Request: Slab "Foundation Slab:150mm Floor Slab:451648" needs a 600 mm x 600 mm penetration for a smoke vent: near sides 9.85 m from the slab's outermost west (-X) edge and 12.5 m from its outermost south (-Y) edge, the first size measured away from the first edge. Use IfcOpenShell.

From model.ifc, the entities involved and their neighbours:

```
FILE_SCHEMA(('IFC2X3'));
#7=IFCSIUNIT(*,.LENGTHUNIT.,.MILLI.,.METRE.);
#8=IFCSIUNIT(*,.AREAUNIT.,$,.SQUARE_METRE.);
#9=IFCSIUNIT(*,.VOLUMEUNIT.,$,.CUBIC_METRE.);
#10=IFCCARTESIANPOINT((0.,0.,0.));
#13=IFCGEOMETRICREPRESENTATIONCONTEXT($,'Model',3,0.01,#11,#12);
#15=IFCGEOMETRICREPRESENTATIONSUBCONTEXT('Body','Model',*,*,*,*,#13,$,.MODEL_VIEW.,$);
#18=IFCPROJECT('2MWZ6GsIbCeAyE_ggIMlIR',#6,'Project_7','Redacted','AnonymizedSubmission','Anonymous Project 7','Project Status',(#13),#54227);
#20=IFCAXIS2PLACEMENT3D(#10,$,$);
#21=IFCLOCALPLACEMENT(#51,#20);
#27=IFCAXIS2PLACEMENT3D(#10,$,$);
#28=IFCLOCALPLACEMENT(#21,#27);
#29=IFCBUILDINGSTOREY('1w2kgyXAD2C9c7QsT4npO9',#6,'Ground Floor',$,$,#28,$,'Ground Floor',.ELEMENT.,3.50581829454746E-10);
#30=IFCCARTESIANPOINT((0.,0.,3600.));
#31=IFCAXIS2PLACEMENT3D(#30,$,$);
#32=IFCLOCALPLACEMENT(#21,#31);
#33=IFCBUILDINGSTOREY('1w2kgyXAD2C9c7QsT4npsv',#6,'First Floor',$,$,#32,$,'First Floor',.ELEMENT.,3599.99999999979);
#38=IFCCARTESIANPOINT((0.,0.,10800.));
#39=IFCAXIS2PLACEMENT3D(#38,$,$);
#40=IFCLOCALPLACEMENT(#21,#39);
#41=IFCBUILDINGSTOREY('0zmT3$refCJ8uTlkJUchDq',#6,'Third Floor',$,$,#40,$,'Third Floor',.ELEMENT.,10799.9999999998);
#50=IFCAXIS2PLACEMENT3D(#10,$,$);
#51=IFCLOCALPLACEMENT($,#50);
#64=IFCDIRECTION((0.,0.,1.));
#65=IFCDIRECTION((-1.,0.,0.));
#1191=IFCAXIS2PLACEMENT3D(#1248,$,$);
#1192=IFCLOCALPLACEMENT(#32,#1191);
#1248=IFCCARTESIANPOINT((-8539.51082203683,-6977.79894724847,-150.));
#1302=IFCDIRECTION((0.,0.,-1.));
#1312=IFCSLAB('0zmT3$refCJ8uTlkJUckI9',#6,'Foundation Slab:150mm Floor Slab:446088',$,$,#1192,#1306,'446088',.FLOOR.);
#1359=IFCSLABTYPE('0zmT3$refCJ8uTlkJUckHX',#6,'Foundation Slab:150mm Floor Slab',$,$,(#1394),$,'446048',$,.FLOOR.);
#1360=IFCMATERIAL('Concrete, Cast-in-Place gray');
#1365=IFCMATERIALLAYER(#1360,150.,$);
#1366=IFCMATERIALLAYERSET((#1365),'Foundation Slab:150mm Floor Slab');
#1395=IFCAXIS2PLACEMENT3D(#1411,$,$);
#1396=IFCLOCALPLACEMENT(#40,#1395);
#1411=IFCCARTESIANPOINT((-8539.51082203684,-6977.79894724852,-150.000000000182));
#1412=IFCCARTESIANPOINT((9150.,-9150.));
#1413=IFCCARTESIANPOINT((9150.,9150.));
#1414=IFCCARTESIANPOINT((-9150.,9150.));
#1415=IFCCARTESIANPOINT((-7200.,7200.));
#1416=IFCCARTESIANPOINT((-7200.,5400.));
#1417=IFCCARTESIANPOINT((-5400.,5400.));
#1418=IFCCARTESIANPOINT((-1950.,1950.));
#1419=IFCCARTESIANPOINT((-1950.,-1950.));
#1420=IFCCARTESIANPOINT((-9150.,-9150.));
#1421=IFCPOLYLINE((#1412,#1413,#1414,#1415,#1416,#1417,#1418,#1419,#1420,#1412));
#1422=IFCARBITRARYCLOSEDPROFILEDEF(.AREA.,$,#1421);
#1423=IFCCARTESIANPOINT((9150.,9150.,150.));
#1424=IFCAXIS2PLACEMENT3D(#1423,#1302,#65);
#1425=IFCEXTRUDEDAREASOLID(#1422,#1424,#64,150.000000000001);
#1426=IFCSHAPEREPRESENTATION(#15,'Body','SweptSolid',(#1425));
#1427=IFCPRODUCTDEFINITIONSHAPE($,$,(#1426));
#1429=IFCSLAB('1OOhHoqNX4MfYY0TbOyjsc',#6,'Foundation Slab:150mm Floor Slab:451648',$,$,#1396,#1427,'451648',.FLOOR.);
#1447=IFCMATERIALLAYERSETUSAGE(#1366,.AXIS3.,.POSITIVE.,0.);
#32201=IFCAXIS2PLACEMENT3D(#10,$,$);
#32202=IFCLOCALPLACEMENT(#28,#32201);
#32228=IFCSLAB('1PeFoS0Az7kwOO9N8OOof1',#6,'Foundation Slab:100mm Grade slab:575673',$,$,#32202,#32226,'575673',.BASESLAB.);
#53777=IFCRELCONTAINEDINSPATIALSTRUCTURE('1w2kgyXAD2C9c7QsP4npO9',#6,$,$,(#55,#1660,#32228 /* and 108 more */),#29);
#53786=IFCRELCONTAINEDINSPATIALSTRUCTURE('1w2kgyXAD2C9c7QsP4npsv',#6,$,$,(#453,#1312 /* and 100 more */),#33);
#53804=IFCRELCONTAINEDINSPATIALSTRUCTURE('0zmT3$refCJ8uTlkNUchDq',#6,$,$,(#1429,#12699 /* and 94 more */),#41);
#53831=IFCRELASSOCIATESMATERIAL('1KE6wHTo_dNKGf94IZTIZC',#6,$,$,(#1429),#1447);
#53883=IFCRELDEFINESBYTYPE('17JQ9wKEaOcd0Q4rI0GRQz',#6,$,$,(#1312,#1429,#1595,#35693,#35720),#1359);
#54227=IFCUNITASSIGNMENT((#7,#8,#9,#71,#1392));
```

```python
import numpy as np
import ifcopenshell
import ifcopenshell.api.feature
import ifcopenshell.api.geometry
import ifcopenshell.api.root
import ifcopenshell.geom
import ifcopenshell.util.placement
import ifcopenshell.util.representation
import ifcopenshell.util.shape
import ifcopenshell.util.unit

model = ifcopenshell.open("model.ifc")
unit_scale = ifcopenshell.util.unit.calculate_unit_scale(model)
settings = ifcopenshell.geom.settings()


def volume(element):
    """Net volume in cubic metres, openings subtracted."""
    shape = ifcopenshell.geom.create_shape(settings, element)
    return ifcopenshell.util.shape.get_volume(shape.geometry)


slab = model.by_id(1429)
before = volume(slab)

# Extent in the slab's own axes, in metres. The edges named are its -X and -Y sides.
slab_shape = ifcopenshell.geom.create_shape(settings, slab)
vertices = ifcopenshell.util.shape.get_vertices(slab_shape.geometry)
x_min, y_min, bottom = vertices.min(axis=0)
top = vertices[:, 2].max()

opening = ifcopenshell.api.root.create_entity(model, ifc_class="IfcOpeningElement", name="Smoke vent opening")
context = ifcopenshell.util.representation.get_context(model, "Model", "Body", "MODEL_VIEW")
width, depth = 0.6, 0.6
outline = [(0.0, 0.0), (width, 0.0), (width, depth), (0.0, depth), (0.0, 0.0)]
# Overshoot both faces by 50 mm so the cut is clean.
shape = ifcopenshell.api.geometry.add_slab_representation(
    model, context=context, depth=top - bottom + 0.1, polyline=outline
)
ifcopenshell.api.geometry.assign_representation(model, product=opening, representation=shape)

matrix = ifcopenshell.util.placement.get_local_placement(slab.ObjectPlacement)
matrix[:, 3] = matrix @ np.append(np.array([x_min + 9.85, y_min + 12.5, bottom - 0.05]) / unit_scale, 1.0)
ifcopenshell.api.geometry.edit_object_placement(model, product=opening, matrix=matrix, is_si=False)
ifcopenshell.api.feature.add_feature(model, feature=opening, element=slab)

after = volume(slab)

print(f"slab volume {before:.3f} -> {after:.3f} m3")

model.write("model_updated.ifc")
```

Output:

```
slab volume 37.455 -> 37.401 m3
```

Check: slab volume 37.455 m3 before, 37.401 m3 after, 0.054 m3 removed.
